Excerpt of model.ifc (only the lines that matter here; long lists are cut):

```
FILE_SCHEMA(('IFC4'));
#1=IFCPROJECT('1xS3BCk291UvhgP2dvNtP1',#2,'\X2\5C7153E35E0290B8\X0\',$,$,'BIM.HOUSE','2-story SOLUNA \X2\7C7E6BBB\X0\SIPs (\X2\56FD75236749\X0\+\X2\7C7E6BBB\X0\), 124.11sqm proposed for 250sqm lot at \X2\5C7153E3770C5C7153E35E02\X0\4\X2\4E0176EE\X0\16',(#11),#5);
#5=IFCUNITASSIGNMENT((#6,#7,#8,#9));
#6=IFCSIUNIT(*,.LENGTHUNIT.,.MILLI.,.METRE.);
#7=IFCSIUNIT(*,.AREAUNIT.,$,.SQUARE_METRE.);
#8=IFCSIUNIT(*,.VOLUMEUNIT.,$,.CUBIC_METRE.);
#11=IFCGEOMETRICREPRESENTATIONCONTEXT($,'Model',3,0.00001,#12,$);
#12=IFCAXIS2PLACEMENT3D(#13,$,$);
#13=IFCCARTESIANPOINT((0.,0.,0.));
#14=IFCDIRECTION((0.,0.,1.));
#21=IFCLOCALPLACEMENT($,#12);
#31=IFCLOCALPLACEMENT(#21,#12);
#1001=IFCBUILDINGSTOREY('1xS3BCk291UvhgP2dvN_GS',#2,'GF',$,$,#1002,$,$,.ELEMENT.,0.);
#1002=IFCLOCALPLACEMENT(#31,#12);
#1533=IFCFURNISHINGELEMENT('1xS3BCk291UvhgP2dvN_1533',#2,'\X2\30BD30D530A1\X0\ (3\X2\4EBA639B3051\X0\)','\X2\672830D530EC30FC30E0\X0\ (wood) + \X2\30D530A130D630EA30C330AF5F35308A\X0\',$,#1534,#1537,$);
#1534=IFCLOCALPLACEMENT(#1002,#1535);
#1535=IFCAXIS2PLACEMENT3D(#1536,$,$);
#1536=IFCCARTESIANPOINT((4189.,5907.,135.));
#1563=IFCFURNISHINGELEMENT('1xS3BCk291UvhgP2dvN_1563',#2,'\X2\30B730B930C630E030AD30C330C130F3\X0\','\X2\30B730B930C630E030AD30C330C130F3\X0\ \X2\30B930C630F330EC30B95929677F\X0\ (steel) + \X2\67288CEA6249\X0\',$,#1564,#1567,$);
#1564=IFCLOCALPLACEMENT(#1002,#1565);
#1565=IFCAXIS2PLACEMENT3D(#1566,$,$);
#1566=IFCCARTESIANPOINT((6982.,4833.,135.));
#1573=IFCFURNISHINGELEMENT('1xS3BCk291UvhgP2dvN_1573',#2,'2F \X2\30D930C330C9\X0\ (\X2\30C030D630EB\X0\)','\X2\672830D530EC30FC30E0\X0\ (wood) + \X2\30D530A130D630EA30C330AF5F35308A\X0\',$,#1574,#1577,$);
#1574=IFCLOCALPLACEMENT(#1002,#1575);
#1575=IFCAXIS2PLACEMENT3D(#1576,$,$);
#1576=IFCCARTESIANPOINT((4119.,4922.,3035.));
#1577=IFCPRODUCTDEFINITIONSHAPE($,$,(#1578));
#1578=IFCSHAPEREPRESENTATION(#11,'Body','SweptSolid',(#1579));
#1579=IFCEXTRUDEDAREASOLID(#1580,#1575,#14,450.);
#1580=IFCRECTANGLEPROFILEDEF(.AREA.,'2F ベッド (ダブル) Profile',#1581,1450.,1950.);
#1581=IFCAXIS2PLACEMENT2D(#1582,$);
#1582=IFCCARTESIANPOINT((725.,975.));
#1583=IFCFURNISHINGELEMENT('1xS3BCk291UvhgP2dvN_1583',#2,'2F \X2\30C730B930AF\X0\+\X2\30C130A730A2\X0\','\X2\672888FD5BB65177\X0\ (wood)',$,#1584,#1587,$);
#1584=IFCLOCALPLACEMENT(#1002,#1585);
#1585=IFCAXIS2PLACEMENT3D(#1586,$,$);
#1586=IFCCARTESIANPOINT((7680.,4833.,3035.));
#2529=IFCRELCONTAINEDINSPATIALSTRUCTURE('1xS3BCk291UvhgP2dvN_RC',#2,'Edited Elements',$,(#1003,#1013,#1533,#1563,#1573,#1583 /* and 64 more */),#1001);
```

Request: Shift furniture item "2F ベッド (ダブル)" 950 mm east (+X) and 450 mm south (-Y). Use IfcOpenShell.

```python
import ifcopenshell
import ifcopenshell.api.geometry
import ifcopenshell.util.placement
import ifcopenshell.util.unit

model = ifcopenshell.open("model.ifc")
unit_scale = ifcopenshell.util.unit.calculate_unit_scale(model)

item = model.by_guid("1xS3BCk291UvhgP2dvN_1573")
matrix = ifcopenshell.util.placement.get_local_placement(item.ObjectPlacement)
matrix[0, 3] += 0.95 / unit_scale
matrix[1, 3] -= 0.45 / unit_scale
ifcopenshell.api.geometry.edit_object_placement(model, product=item, matrix=matrix, is_si=False)

print(ifcopenshell.util.placement.get_local_placement(item.ObjectPlacement).round(3) + 0.0)

model.write("model_updated.ifc")
```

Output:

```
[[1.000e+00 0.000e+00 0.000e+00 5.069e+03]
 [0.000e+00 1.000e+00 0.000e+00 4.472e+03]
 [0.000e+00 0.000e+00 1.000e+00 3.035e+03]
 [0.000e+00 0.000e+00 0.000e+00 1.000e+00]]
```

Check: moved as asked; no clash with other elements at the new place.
